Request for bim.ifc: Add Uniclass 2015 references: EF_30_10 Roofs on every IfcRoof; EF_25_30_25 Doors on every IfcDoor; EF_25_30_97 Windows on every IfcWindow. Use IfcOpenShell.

First a look at what the model holds.

```python
import ifcopenshell

model = ifcopenshell.open("bim.ifc")
print(model.schema)
print("classifications:", [c.Name for c in model.by_type("IfcClassification")])
for ifc_class in ("IfcDoor", "IfcRoof", "IfcStair", "IfcWall", "IfcWindow"):
    print(ifc_class, len(model.by_type(ifc_class)))
```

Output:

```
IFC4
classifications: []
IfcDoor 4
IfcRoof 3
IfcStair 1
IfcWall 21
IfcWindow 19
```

```python
import ifcopenshell
import ifcopenshell.api.classification

model = ifcopenshell.open("bim.ifc")

system = ifcopenshell.api.classification.add_classification(model, classification="Uniclass 2015")

codes = {
    "IfcRoof": ("EF_30_10", "Roofs"),
    "IfcDoor": ("EF_25_30_25", "Doors"),
    "IfcWindow": ("EF_25_30_97", "Windows"),
}
for ifc_class, (code, name) in codes.items():
    products = model.by_type(ifc_class)
    ifcopenshell.api.classification.add_reference(
        model, products=products, classification=system, identification=code, name=name
    )
    print(code, len(products))

model.write("bim_v2.ifc")
```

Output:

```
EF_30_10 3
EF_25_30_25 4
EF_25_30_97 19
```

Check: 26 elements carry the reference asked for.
